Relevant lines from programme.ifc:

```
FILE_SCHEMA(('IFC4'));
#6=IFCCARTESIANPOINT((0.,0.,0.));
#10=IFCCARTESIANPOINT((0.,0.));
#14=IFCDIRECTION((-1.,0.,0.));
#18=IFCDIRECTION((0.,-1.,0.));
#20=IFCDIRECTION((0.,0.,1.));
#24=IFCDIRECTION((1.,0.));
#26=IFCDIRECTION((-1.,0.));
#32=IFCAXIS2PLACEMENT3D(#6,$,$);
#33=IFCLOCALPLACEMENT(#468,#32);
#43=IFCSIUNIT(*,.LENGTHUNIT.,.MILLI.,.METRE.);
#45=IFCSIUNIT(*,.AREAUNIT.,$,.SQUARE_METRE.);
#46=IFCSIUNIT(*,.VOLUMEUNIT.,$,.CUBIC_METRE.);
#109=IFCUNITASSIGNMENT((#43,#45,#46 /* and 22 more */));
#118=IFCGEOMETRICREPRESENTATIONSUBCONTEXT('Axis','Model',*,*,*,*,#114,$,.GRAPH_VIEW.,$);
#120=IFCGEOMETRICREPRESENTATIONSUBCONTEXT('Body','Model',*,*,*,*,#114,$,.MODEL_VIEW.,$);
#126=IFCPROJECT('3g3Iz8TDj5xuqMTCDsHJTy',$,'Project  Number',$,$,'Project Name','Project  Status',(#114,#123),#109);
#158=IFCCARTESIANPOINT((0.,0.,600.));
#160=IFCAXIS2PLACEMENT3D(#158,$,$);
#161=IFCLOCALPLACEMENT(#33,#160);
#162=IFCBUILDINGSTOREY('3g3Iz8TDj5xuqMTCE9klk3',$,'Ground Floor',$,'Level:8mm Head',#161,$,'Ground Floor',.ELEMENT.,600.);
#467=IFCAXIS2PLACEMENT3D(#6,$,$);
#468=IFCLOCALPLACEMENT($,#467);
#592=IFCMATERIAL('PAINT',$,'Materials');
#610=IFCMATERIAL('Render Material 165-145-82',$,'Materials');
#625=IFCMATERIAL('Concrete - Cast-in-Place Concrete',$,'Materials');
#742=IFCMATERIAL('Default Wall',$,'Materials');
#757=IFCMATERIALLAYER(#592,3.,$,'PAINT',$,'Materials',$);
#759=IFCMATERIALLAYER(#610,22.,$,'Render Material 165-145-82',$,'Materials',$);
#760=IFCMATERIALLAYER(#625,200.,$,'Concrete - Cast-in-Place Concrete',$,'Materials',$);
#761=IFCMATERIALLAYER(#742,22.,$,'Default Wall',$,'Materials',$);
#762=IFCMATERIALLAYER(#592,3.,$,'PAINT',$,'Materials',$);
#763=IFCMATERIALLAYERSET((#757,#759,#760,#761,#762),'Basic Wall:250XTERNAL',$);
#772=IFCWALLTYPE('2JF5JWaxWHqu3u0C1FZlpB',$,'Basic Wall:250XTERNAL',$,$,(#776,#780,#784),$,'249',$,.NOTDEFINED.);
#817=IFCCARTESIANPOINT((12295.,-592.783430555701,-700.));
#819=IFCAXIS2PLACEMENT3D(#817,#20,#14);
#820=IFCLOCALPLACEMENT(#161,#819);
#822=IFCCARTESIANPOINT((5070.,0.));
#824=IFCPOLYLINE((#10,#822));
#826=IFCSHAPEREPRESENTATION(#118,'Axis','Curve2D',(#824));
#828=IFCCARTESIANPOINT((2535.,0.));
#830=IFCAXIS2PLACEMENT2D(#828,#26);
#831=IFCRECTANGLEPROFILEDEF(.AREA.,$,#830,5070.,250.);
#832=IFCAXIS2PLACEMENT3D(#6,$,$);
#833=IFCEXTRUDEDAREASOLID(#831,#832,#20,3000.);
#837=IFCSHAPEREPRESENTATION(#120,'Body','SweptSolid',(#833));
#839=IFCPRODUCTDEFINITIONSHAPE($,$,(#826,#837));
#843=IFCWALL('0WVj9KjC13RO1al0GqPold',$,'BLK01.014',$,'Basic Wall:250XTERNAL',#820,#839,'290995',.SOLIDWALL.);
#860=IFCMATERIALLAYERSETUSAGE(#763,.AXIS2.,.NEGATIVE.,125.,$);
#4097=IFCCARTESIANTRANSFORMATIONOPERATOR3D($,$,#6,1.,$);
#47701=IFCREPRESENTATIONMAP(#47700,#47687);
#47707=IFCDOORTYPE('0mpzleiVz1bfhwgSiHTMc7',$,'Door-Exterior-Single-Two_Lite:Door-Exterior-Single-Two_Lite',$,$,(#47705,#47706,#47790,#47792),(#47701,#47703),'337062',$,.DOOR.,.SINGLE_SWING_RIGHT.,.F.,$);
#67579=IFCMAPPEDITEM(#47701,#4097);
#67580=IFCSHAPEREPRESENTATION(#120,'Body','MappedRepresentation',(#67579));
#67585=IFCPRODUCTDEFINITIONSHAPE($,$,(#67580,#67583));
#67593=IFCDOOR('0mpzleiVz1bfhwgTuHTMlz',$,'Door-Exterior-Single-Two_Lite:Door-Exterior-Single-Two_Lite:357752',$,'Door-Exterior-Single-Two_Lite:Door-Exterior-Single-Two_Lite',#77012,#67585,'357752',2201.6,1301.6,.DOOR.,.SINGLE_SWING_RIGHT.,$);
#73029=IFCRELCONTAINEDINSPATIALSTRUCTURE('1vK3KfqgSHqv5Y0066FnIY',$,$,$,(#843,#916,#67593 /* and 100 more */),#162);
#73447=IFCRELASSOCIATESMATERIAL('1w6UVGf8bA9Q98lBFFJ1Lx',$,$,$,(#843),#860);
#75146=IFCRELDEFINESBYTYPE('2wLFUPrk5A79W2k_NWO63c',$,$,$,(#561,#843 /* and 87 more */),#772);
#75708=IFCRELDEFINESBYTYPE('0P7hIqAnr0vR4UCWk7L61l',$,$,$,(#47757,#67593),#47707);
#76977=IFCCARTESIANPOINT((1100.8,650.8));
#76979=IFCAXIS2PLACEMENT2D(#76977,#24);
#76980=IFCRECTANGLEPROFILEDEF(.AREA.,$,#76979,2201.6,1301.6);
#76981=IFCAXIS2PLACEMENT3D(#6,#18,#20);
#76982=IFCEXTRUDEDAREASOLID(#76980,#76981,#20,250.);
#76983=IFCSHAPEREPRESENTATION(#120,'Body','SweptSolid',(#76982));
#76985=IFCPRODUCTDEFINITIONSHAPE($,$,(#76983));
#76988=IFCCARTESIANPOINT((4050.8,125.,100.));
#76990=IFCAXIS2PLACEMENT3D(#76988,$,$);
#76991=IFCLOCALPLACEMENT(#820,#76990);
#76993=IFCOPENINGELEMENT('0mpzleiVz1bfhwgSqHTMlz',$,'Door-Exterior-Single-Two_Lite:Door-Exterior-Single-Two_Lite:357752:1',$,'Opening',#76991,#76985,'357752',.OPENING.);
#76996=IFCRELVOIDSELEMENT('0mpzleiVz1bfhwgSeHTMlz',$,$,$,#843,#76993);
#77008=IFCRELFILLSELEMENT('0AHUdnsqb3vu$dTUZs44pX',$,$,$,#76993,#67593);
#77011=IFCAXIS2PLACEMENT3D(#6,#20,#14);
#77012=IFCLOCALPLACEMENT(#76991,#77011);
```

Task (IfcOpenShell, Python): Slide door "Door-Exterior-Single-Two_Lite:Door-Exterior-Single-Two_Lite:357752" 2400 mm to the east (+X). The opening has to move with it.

```python
import ifcopenshell
import ifcopenshell.api.geometry
import ifcopenshell.util.placement
import ifcopenshell.util.unit

model = ifcopenshell.open("programme.ifc")
unit_scale = ifcopenshell.util.unit.calculate_unit_scale(model)

door = model.by_guid("0mpzleiVz1bfhwgTuHTMlz")
opening = door.FillsVoids[0].RelatingOpeningElement
wall = opening.VoidsElements[0].RelatingBuildingElement

wall_matrix = ifcopenshell.util.placement.get_local_placement(wall.ObjectPlacement)
shift = wall_matrix[:3, 0] * -2.4 / unit_scale
before = ifcopenshell.util.placement.get_local_placement(door.ObjectPlacement)[:3, 3].copy()

# The door is placed relative to its opening, so it follows when the opening moves.
matrix = ifcopenshell.util.placement.get_local_placement(opening.ObjectPlacement)
matrix[:3, 3] += shift
ifcopenshell.api.geometry.edit_object_placement(
    model, product=opening, matrix=matrix, is_si=False, should_transform_children=True
)

after = ifcopenshell.util.placement.get_local_placement(door.ObjectPlacement)[:3, 3]
print("door moved by", (after - before).round(3) + 0.0)

model.write("programme_rev.ifc")
```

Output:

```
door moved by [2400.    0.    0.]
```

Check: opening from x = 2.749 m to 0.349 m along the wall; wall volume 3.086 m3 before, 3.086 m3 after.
